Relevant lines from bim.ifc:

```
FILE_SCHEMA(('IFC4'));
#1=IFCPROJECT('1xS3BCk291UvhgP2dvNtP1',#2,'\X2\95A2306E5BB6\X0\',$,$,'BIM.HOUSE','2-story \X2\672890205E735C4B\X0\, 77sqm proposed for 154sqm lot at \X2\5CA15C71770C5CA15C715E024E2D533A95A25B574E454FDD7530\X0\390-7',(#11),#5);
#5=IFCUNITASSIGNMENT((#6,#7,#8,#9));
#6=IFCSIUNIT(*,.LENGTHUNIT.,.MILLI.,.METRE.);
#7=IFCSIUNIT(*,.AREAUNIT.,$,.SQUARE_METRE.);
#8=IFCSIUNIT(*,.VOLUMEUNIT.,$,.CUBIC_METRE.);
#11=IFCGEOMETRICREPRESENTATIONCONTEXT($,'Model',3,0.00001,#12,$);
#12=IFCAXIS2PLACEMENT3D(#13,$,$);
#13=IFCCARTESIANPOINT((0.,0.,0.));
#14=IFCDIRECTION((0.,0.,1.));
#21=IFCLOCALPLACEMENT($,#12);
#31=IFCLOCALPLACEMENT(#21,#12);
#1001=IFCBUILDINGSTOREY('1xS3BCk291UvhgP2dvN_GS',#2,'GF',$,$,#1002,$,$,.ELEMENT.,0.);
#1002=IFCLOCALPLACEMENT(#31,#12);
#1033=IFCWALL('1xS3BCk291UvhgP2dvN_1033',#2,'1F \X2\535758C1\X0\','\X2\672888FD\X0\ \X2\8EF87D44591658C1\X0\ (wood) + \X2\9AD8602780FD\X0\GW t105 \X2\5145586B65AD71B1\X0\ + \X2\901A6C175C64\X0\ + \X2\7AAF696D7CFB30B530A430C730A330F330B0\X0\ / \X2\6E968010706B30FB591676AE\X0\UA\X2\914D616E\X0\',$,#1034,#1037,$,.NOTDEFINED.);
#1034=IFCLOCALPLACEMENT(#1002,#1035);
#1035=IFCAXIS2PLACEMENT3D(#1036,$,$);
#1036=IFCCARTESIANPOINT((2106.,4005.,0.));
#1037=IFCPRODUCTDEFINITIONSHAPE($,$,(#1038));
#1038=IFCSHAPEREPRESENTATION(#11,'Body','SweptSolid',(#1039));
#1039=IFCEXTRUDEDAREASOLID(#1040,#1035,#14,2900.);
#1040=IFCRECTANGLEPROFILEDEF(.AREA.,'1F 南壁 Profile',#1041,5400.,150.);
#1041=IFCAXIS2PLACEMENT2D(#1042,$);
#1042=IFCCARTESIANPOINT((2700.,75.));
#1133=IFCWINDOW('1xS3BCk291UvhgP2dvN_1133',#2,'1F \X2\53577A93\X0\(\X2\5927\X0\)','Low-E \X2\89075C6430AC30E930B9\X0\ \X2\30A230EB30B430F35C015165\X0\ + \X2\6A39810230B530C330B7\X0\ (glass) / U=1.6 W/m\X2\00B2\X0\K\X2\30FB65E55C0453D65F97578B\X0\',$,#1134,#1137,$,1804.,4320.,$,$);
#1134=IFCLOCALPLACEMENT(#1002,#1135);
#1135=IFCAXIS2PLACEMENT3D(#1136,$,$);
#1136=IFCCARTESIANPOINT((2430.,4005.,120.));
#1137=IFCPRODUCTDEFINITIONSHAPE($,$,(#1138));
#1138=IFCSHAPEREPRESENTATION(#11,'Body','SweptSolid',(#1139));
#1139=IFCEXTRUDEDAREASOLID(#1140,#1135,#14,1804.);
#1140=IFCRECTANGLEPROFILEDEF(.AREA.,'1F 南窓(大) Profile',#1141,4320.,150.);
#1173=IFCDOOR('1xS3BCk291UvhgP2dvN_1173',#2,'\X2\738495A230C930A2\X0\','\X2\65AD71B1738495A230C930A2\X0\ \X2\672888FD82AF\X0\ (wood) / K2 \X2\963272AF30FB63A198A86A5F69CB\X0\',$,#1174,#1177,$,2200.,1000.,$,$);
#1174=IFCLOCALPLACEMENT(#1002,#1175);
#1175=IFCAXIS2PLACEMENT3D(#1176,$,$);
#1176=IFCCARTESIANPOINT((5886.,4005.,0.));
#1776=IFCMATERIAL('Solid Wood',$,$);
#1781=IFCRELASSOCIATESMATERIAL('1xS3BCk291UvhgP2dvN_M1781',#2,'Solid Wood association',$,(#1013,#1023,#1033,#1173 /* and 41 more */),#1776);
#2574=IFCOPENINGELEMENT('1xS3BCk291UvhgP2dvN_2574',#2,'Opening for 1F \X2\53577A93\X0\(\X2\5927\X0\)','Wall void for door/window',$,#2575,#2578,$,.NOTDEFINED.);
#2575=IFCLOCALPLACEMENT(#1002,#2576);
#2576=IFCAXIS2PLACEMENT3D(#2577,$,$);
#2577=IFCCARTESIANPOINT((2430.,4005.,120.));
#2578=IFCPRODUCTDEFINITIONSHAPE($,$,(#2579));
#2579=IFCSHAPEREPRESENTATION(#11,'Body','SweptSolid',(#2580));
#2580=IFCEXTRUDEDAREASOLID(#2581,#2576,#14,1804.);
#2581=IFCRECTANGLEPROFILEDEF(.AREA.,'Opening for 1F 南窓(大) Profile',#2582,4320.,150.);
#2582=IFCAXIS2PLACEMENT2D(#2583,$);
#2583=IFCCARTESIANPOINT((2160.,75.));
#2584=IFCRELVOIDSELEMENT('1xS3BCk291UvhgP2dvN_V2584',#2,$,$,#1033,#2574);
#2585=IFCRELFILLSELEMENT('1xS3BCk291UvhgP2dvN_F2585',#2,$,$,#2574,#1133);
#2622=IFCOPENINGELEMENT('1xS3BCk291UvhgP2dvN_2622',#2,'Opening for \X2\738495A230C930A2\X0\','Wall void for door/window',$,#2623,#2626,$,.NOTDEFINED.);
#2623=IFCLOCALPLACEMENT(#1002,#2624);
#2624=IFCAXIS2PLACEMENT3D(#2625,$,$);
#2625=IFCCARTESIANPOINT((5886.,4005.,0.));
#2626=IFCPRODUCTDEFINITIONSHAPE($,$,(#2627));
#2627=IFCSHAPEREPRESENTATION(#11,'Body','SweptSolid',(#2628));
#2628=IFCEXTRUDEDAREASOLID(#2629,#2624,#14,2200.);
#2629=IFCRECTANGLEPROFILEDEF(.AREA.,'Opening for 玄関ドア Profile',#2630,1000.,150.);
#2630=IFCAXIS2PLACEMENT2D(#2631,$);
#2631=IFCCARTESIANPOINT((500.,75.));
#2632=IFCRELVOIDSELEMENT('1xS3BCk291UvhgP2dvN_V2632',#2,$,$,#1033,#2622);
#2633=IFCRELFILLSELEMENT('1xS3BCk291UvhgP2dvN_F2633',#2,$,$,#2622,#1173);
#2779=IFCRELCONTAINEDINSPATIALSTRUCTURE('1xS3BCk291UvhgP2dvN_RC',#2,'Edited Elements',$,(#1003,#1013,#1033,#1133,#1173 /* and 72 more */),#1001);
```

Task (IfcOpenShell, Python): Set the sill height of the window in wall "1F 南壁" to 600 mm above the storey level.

```python
import numpy as np
import ifcopenshell
import ifcopenshell.api.geometry
import ifcopenshell.geom
import ifcopenshell.util.element
import ifcopenshell.util.placement
import ifcopenshell.util.shape
import ifcopenshell.util.unit

model = ifcopenshell.open("bim.ifc")
unit_scale = ifcopenshell.util.unit.calculate_unit_scale(model)

window = model.by_id(1133)
opening = window.FillsVoids[0].RelatingOpeningElement
storey = ifcopenshell.util.element.get_container(window, ifc_class="IfcBuildingStorey")
level = ifcopenshell.util.placement.get_local_placement(storey.ObjectPlacement)[2, 3]

# The opening's origin need not be at the sill, so measure its lowest point.
shape = ifcopenshell.geom.create_shape(ifcopenshell.geom.settings(), opening)
bottom = ifcopenshell.util.shape.get_shape_bottom_elevation(shape, shape.geometry) / unit_scale
dz = level + 0.6 / unit_scale - bottom

shift = np.array([0.0, 0.0, dz])
# The window is not placed relative to its opening, so move both.
for product in (opening, window):
    matrix = ifcopenshell.util.placement.get_local_placement(product.ObjectPlacement)
    matrix[:3, 3] += shift
    ifcopenshell.api.geometry.edit_object_placement(model, product=product, matrix=matrix, is_si=False)

print(f"moved by {dz * unit_scale:+.3f} m")

model.write("bim-out.ifc")
```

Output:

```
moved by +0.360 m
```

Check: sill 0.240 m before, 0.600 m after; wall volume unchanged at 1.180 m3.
